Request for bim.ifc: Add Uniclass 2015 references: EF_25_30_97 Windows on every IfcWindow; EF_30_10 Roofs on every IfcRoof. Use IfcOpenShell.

First a look at what the model holds.

```python
import ifcopenshell

model = ifcopenshell.open("bim.ifc")
print(model.schema)
print("classifications:", [c.Name for c in model.by_type("IfcClassification")])
for ifc_class in ("IfcDoor", "IfcRoof", "IfcStair", "IfcWall", "IfcWindow"):
    print(ifc_class, len(model.by_type(ifc_class)))
```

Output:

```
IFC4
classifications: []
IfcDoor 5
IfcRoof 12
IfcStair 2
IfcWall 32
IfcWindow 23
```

```python
import ifcopenshell
import ifcopenshell.api.classification

model = ifcopenshell.open("bim.ifc")

system = ifcopenshell.api.classification.add_classification(model, classification="Uniclass 2015")

codes = {
    "IfcWindow": ("EF_25_30_97", "Windows"),
    "IfcRoof": ("EF_30_10", "Roofs"),
}
for ifc_class, (code, name) in codes.items():
    products = model.by_type(ifc_class)
    ifcopenshell.api.classification.add_reference(
        model, products=products, classification=system, identification=code, name=name
    )
    print(code, len(products))

model.write("bim_rev.ifc")
```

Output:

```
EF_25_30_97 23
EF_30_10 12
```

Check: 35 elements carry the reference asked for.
